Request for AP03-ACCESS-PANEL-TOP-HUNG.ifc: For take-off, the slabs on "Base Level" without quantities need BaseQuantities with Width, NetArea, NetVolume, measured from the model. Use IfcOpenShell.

First a look at what the model holds.

```python
import ifcopenshell
import ifcopenshell.util.element
import ifcopenshell.util.unit

model = ifcopenshell.open("AP03-ACCESS-PANEL-TOP-HUNG.ifc")
print(model.schema)
for unit_type in ("LENGTHUNIT", "AREAUNIT", "VOLUMEUNIT"):
    print(unit_type, ifcopenshell.util.unit.calculate_unit_scale(model, unit_type))
storey = next(s for s in model.by_type("IfcBuildingStorey") if s.Name == "Base Level")
slabs = [e for e in ifcopenshell.util.element.get_decomposition(storey) if e.is_a("IfcSlab")]
for e in sorted(slabs, key=lambda e: e.id()):
    print(e.id(), e.is_a(), e.Name, list(ifcopenshell.util.element.get_psets(e, qtos_only=True)), sep=" | ")
```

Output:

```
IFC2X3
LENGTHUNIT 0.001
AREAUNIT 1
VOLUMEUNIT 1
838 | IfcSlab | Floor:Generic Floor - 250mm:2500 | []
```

```python
import ifcopenshell
import ifcopenshell.api.pset
import ifcopenshell.geom
import ifcopenshell.util.element
import ifcopenshell.util.shape
import ifcopenshell.util.unit

model = ifcopenshell.open("AP03-ACCESS-PANEL-TOP-HUNG.ifc")
unit_scale = ifcopenshell.util.unit.calculate_unit_scale(model)
area_scale = ifcopenshell.util.unit.calculate_unit_scale(model, "AREAUNIT")
volume_scale = ifcopenshell.util.unit.calculate_unit_scale(model, "VOLUMEUNIT")
settings = ifcopenshell.geom.settings()

storey = next(s for s in model.by_type("IfcBuildingStorey") if s.Name == "Base Level")
slabs = [e for e in ifcopenshell.util.element.get_decomposition(storey) if e.is_a("IfcSlab")]

for e in sorted(slabs, key=lambda e: e.id()):
    if ifcopenshell.util.element.get_psets(e, qtos_only=True, should_inherit=False):
        continue
    # Geometry comes back in metres, in the element's own axes.
    shape = ifcopenshell.geom.create_shape(settings, e)
    values = {
        "Width": ifcopenshell.util.shape.get_z(shape.geometry) / unit_scale,
        "NetArea": ifcopenshell.util.shape.get_footprint_area(shape.geometry) / area_scale,
        "NetVolume": ifcopenshell.util.shape.get_volume(shape.geometry) / volume_scale,
    }
    qto = ifcopenshell.api.pset.add_qto(model, product=e, name="BaseQuantities")
    ifcopenshell.api.pset.edit_qto(model, qto=qto, properties=values)
    print(e.id(), {k: round(v, 3) for k, v in values.items()})

model.write("AP03-ACCESS-PANEL-TOP-HUNG_updated.ifc")
```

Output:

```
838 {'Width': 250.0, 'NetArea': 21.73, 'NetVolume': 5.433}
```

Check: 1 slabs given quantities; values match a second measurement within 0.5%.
